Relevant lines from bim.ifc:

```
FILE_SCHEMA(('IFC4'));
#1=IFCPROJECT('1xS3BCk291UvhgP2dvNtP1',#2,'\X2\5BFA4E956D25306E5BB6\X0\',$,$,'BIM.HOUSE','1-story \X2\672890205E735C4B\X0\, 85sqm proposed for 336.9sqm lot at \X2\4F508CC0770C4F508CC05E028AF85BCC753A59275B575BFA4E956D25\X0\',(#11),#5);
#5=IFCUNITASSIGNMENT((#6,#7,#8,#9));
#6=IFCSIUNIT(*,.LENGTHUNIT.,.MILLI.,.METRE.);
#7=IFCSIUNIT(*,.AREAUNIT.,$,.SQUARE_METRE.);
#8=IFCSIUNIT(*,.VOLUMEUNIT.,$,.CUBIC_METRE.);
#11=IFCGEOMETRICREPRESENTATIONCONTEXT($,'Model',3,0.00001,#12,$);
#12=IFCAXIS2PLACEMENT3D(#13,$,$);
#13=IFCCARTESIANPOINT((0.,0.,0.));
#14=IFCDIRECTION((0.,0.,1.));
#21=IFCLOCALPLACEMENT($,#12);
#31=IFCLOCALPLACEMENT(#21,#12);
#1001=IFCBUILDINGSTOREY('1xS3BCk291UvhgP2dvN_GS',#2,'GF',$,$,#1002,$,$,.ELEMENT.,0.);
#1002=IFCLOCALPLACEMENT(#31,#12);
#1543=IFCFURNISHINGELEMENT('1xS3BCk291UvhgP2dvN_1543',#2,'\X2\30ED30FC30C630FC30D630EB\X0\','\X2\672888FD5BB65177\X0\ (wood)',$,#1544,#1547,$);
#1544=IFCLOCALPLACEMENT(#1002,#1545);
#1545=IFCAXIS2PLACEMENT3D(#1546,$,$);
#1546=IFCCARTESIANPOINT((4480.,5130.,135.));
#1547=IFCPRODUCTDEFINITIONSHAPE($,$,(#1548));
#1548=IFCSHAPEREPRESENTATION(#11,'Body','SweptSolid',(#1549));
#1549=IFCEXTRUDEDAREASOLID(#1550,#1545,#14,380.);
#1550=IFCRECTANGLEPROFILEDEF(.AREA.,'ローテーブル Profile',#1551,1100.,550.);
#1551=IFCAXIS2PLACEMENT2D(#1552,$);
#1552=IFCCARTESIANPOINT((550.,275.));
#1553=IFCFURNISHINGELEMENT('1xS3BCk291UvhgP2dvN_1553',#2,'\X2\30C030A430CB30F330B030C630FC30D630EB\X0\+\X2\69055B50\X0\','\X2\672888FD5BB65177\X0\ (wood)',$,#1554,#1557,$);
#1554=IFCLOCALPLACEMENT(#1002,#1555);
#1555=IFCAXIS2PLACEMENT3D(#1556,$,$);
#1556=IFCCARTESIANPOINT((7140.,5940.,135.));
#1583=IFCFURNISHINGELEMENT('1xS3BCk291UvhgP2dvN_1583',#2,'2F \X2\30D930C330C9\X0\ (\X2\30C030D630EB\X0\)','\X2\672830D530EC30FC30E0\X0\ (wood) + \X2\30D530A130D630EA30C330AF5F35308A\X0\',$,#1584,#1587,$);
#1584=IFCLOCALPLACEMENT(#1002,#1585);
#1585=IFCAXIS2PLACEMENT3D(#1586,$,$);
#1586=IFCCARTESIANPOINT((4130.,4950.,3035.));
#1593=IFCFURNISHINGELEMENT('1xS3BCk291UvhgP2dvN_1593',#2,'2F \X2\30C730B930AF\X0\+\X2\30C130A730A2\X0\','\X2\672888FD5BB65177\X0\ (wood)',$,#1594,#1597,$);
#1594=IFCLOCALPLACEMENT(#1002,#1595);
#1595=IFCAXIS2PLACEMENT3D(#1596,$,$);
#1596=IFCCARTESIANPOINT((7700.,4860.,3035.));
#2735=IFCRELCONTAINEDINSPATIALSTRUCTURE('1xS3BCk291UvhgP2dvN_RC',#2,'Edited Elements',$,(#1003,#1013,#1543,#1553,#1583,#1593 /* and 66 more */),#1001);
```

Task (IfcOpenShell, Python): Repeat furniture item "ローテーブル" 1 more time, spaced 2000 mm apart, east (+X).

```python
import numpy as np
import ifcopenshell
import ifcopenshell.api.geometry
import ifcopenshell.api.root
import ifcopenshell.util.element
import ifcopenshell.util.placement
import ifcopenshell.util.unit

model = ifcopenshell.open("bim.ifc")
unit_scale = ifcopenshell.util.unit.calculate_unit_scale(model)


def reuse_history(source, copy):
    """copy_class also copies each property set's owner history, people and application; keep the originals."""
    for rel in copy.IsDefinedBy:
        if rel.is_a("IfcRelDefinesByProperties") and (history := rel.RelatingPropertyDefinition.OwnerHistory):
            rel.RelatingPropertyDefinition.OwnerHistory = source.OwnerHistory
            ifcopenshell.util.element.remove_deep2(model, history)


source = model.by_guid("1xS3BCk291UvhgP2dvN_1543")
base = ifcopenshell.util.placement.get_local_placement(source.ObjectPlacement)
step = np.array([1.0, 0.0, 0.0]) * 2 / unit_scale

for i in range(1, 2):
    copy = ifcopenshell.api.root.copy_class(model, product=source)
    copy.Representation = ifcopenshell.util.element.copy_deep(
        model, source.Representation, exclude=["IfcGeometricRepresentationContext", "IfcRepresentationMap"]
    )
    reuse_history(source, copy)
    matrix = base.copy()
    matrix[:3, 3] += i * step
    print("added at", matrix[:3, 3].round(3) + 0.0)
    ifcopenshell.api.geometry.edit_object_placement(model, product=copy, matrix=matrix, is_si=False)

model.write("bim-out.ifc")
```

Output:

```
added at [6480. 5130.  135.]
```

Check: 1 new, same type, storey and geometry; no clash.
